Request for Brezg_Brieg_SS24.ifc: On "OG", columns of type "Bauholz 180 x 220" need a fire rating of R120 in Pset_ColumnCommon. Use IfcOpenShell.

First a look at what the model holds.

```python
import ifcopenshell
import ifcopenshell.util.element

model = ifcopenshell.open("Brezg_Brieg_SS24.ifc")
print(model.schema)
storey = next(s for s in model.by_type("IfcBuildingStorey") if s.Name == "OG")
columns = [e for e in ifcopenshell.util.element.get_decomposition(storey) if e.is_a("IfcColumn")]
seen = {}
for e in columns:
    element_type = ifcopenshell.util.element.get_type(e)
    key = (element_type.Name if element_type != e and element_type else None, ifcopenshell.util.element.get_pset(e, "Pset_ColumnCommon", "FireRating"))
    seen[key] = seen.get(key, 0) + 1
for (name, value), count in sorted(seen.items(), key=str):
    print(count, "x", name, "|", value)
```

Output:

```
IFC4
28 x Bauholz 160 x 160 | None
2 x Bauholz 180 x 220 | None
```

```python
import ifcopenshell
import ifcopenshell.api.pset
import ifcopenshell.util.element

model = ifcopenshell.open("Brezg_Brieg_SS24.ifc")

storey = next(s for s in model.by_type("IfcBuildingStorey") if s.Name == "OG")
columns = [e for e in ifcopenshell.util.element.get_decomposition(storey) if e.is_a("IfcColumn")]

count = 0
for e in columns:
    element_type = ifcopenshell.util.element.get_type(e)
    if element_type in (None, e) or element_type.Name != "Bauholz 180 x 220":
        continue
    # add_pset returns the element's existing set when there is one.
    pset = ifcopenshell.api.pset.add_pset(model, product=e, name="Pset_ColumnCommon")
    ifcopenshell.api.pset.edit_pset(model, pset=pset, properties={"FireRating": "R120"})
    count += 1

print(count, "columns updated")

model.write("Brezg_Brieg_SS24-out.ifc")
```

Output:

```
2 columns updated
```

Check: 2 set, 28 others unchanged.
